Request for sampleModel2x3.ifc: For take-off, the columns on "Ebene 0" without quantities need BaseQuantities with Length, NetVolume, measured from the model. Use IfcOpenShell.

First a look at what the model holds.

```python
import ifcopenshell
import ifcopenshell.util.element
import ifcopenshell.util.unit

model = ifcopenshell.open("sampleModel2x3.ifc")
print(model.schema)
for unit_type in ("LENGTHUNIT", "AREAUNIT", "VOLUMEUNIT"):
    print(unit_type, ifcopenshell.util.unit.calculate_unit_scale(model, unit_type))
storey = next(s for s in model.by_type("IfcBuildingStorey") if s.Name == "Ebene 0")
columns = [e for e in ifcopenshell.util.element.get_decomposition(storey) if e.is_a("IfcColumn")]
for e in sorted(columns, key=lambda e: e.id()):
    print(e.id(), e.is_a(), e.Name, list(ifcopenshell.util.element.get_psets(e, qtos_only=True)), sep=" | ")
```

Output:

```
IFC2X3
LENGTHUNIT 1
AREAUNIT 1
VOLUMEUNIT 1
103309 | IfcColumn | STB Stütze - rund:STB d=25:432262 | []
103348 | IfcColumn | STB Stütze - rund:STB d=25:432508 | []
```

```python
import ifcopenshell
import ifcopenshell.api.pset
import ifcopenshell.geom
import ifcopenshell.util.element
import ifcopenshell.util.shape
import ifcopenshell.util.unit

model = ifcopenshell.open("sampleModel2x3.ifc")
unit_scale = ifcopenshell.util.unit.calculate_unit_scale(model)
volume_scale = ifcopenshell.util.unit.calculate_unit_scale(model, "VOLUMEUNIT")
settings = ifcopenshell.geom.settings()

storey = next(s for s in model.by_type("IfcBuildingStorey") if s.Name == "Ebene 0")
columns = [e for e in ifcopenshell.util.element.get_decomposition(storey) if e.is_a("IfcColumn")]

for e in sorted(columns, key=lambda e: e.id()):
    if ifcopenshell.util.element.get_psets(e, qtos_only=True, should_inherit=False):
        continue
    # Geometry comes back in metres, in the element's own axes.
    shape = ifcopenshell.geom.create_shape(settings, e)
    values = {
        "Length": ifcopenshell.util.shape.get_z(shape.geometry) / unit_scale,
        "NetVolume": ifcopenshell.util.shape.get_volume(shape.geometry) / volume_scale,
    }
    qto = ifcopenshell.api.pset.add_qto(model, product=e, name="BaseQuantities")
    ifcopenshell.api.pset.edit_qto(model, qto=qto, properties=values)
    print(e.id(), {k: round(v, 3) for k, v in values.items()})

model.write("sampleModel2x3_v2.ifc")
```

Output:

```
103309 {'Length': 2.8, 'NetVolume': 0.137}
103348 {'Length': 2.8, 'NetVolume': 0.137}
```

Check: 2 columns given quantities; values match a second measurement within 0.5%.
